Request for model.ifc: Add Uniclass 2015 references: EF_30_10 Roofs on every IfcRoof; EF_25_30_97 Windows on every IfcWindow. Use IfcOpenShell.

First a look at what the model holds.

```python
import ifcopenshell

model = ifcopenshell.open("model.ifc")
print(model.schema)
print("classifications:", [c.Name for c in model.by_type("IfcClassification")])
for ifc_class in ("IfcDoor", "IfcRoof", "IfcStair", "IfcWall", "IfcWindow"):
    print(ifc_class, len(model.by_type(ifc_class)))
```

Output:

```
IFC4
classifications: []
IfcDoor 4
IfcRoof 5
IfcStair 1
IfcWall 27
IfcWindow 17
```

```python
import ifcopenshell
import ifcopenshell.api.classification

model = ifcopenshell.open("model.ifc")

system = ifcopenshell.api.classification.add_classification(model, classification="Uniclass 2015")

codes = {
    "IfcRoof": ("EF_30_10", "Roofs"),
    "IfcWindow": ("EF_25_30_97", "Windows"),
}
for ifc_class, (code, name) in codes.items():
    products = model.by_type(ifc_class)
    ifcopenshell.api.classification.add_reference(
        model, products=products, classification=system, identification=code, name=name
    )
    print(code, len(products))

model.write("model_updated.ifc")
```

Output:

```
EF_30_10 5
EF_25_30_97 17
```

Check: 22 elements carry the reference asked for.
